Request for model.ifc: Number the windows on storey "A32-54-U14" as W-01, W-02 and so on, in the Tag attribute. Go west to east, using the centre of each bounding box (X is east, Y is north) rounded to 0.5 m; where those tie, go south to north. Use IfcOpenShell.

First a look at what the model holds.

```python
import ifcopenshell
import ifcopenshell.util.element
import ifcopenshell.util.placement

model = ifcopenshell.open("model.ifc")
print(model.schema)
storey = next(s for s in model.by_type("IfcBuildingStorey") if s.Name == "A32-54-U14")
windows = [e for e in ifcopenshell.util.element.get_decomposition(storey) if e.is_a("IfcWindow")]
for e in sorted(windows, key=lambda e: e.id()):
    origin = ifcopenshell.util.placement.get_local_placement(e.ObjectPlacement)[:3, 3]
    print(e.id(), e.Tag, e.Name, origin.round(2) + 0.0, sep=" | ")
```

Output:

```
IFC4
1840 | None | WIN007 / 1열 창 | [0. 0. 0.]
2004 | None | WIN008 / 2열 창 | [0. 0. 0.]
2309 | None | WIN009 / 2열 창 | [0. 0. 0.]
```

```python
import ifcopenshell
import ifcopenshell.geom
import ifcopenshell.util.element
import ifcopenshell.util.shape

model = ifcopenshell.open("model.ifc")
settings = ifcopenshell.geom.settings()
settings.set("use-world-coords", True)


def centre(element):
    shape = ifcopenshell.geom.create_shape(settings, element)
    return ifcopenshell.util.shape.get_bbox_centroid(shape.geometry)


storey = next(s for s in model.by_type("IfcBuildingStorey") if s.Name == "A32-54-U14")
windows = [e for e in ifcopenshell.util.element.get_decomposition(storey) if e.is_a("IfcWindow")]

# Insertion points can sit at a corner or the storey origin, so sort by the geometry (in metres).
centres = {e: centre(e) for e in windows}
windows.sort(key=lambda e: (round(centres[e][0] / 0.5), centres[e][1]))

for i, e in enumerate(windows, start=1):
    number = f"W-{i:02d}"
    e.Tag = number
    print(e.id(), number)

model.write("model_edited.ifc")
```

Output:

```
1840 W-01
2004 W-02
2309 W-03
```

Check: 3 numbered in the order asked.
